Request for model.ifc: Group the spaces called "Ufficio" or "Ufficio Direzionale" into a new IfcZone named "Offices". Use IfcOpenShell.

First a look at what the model holds.

```python
import ifcopenshell

model = ifcopenshell.open("model.ifc")
print(model.schema)
seen = {}
for space in model.by_type("IfcSpace"):
    seen[space.LongName] = seen.get(space.LongName, 0) + 1
for name, count in sorted(seen.items(), key=str):
    print(count, "x", name)
print("zones:", [z.Name for z in model.by_type("IfcZone")][:20])
```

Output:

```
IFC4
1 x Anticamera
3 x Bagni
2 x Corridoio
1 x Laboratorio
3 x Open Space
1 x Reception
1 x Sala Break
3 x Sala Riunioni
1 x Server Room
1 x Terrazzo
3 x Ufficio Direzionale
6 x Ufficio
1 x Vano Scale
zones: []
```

```python
import ifcopenshell
import ifcopenshell.api.group
import ifcopenshell.api.root

model = ifcopenshell.open("model.ifc")

names = {"Ufficio", "Ufficio Direzionale"}
spaces = [s for s in model.by_type("IfcSpace") if s.LongName in names]

zone = ifcopenshell.api.root.create_entity(model, ifc_class="IfcZone", name="Offices")
ifcopenshell.api.group.assign_group(model, products=spaces, group=zone)
print(len(spaces), "spaces in", zone.Name)

model.write("model_edited.ifc")
```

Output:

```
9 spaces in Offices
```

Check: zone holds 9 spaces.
